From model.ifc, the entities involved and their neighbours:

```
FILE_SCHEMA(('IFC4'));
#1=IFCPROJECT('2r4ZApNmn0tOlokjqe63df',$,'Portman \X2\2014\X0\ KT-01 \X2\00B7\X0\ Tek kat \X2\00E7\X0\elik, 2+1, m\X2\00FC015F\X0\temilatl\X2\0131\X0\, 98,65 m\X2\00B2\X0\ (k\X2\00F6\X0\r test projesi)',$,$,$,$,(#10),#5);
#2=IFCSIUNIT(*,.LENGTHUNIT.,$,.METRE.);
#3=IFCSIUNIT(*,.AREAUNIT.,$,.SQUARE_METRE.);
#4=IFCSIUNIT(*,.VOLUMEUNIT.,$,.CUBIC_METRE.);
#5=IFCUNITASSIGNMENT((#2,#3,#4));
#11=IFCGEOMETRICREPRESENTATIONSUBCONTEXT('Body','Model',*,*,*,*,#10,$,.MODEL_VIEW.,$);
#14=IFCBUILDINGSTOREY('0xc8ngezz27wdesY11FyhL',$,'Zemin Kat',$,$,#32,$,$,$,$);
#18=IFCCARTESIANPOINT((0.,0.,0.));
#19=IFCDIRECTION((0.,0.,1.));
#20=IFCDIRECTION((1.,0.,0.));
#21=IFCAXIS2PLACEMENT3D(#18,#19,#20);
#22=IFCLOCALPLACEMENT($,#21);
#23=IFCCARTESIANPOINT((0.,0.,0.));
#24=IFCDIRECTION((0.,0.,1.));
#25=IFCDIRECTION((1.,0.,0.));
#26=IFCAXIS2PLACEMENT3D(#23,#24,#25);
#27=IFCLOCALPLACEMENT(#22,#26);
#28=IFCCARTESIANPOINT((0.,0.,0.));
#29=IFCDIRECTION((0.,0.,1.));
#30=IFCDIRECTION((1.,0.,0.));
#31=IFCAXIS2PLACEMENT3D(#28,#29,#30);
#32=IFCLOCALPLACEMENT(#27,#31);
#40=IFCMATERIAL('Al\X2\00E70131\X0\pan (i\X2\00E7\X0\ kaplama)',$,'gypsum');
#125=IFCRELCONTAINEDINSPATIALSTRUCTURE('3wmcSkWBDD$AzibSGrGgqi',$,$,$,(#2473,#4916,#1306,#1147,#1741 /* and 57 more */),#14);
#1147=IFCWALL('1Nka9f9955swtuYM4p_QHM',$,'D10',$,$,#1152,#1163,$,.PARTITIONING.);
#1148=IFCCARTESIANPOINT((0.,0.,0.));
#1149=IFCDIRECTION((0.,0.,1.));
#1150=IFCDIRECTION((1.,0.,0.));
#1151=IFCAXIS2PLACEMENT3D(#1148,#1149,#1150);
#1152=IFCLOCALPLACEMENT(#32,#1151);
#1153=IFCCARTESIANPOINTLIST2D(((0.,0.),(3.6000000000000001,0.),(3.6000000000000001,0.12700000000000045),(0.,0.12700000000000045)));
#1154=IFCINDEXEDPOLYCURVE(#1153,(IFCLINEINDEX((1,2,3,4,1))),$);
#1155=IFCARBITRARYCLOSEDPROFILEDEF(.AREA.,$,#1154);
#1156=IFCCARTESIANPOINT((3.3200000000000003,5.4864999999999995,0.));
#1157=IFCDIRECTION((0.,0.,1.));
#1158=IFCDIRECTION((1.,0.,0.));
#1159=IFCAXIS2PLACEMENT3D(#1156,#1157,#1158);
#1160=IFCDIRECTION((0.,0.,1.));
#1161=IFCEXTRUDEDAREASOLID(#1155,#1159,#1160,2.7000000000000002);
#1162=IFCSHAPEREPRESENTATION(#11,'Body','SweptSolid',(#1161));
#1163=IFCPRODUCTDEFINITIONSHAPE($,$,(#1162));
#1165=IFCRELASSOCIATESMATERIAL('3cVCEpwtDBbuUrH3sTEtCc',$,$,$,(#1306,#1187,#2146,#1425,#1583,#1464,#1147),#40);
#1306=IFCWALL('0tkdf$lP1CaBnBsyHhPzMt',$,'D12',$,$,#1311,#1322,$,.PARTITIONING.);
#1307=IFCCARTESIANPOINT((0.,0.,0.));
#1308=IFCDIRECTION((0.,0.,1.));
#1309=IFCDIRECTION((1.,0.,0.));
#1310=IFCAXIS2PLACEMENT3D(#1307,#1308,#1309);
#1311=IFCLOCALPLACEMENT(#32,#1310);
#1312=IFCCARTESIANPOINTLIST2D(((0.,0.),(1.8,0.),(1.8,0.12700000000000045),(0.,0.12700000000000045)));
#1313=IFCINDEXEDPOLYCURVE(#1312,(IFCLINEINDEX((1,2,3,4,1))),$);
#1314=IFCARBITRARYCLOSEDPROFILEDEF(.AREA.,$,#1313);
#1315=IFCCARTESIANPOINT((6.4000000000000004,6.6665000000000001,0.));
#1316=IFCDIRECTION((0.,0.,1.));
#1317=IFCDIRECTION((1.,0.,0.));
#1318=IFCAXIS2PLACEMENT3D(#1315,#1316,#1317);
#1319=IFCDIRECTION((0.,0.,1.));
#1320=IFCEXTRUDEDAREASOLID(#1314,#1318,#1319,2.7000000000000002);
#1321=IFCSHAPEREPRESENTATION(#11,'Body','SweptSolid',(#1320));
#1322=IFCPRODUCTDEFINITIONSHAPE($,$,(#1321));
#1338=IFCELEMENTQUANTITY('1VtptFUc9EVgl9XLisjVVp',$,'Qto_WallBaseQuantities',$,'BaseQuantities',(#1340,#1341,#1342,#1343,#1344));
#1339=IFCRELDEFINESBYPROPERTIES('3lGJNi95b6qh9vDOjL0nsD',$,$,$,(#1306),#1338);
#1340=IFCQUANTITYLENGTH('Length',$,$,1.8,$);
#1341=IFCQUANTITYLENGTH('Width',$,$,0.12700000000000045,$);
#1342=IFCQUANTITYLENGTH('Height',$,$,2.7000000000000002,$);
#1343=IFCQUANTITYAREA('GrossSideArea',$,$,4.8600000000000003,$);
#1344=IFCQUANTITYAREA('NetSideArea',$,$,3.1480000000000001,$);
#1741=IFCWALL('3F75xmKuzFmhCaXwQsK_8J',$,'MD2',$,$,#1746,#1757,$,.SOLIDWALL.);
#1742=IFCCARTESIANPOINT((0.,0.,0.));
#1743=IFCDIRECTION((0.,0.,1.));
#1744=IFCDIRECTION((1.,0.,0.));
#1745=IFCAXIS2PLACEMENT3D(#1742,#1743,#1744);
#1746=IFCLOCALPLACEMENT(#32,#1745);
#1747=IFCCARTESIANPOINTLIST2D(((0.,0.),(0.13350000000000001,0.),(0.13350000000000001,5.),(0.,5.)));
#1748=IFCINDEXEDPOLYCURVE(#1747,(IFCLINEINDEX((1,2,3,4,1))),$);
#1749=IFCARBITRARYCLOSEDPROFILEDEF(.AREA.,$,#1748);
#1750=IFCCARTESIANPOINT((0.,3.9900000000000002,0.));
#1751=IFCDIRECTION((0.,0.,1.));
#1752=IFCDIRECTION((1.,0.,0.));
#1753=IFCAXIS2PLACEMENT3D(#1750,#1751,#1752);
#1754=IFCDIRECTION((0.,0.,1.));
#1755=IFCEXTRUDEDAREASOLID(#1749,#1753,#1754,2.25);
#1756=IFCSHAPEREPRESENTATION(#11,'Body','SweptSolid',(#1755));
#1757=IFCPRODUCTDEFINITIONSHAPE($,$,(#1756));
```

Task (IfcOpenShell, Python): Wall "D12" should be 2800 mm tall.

```python
import ifcopenshell
import ifcopenshell.api.pset
import ifcopenshell.geom
import ifcopenshell.util.element
import ifcopenshell.util.representation
import ifcopenshell.util.shape
import ifcopenshell.util.unit

model = ifcopenshell.open("model.ifc")
unit_scale = ifcopenshell.util.unit.calculate_unit_scale(model)
area_scale = ifcopenshell.util.unit.calculate_unit_scale(model, "AREAUNIT")
settings = ifcopenshell.geom.settings()


def volume(element):
    """Net volume in cubic metres, openings subtracted."""
    shape = ifcopenshell.geom.create_shape(settings, element)
    return ifcopenshell.util.shape.get_volume(shape.geometry)


wall = model.by_id(1306)
before = volume(wall)

body = ifcopenshell.util.representation.get_representation(wall, "Model", "Body")
solid = body.Items[0]
old_height = solid.Depth
solid.Depth = 2.8
after = volume(wall)
thickness = 0.127  # wall thickness in metres

# Update the stored height, areas and volumes.
qto = model.by_id(ifcopenshell.util.element.get_pset(wall, "Qto_WallBaseQuantities", should_inherit=False)["id"])
ifcopenshell.api.pset.edit_qto(model, qto=qto, properties={
    "Height": solid.Depth,
    "GrossSideArea": ifcopenshell.util.element.get_pset(wall, "Qto_WallBaseQuantities", "GrossSideArea") * solid.Depth / old_height,
    "NetSideArea": after / thickness / area_scale,
})

print(f"height {old_height:g} -> {solid.Depth:g}, volume {before:.3f} -> {after:.3f} m3")

model.write("model_v2.ifc")
```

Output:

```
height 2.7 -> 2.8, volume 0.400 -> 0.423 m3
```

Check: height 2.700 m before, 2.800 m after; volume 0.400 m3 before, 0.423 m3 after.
